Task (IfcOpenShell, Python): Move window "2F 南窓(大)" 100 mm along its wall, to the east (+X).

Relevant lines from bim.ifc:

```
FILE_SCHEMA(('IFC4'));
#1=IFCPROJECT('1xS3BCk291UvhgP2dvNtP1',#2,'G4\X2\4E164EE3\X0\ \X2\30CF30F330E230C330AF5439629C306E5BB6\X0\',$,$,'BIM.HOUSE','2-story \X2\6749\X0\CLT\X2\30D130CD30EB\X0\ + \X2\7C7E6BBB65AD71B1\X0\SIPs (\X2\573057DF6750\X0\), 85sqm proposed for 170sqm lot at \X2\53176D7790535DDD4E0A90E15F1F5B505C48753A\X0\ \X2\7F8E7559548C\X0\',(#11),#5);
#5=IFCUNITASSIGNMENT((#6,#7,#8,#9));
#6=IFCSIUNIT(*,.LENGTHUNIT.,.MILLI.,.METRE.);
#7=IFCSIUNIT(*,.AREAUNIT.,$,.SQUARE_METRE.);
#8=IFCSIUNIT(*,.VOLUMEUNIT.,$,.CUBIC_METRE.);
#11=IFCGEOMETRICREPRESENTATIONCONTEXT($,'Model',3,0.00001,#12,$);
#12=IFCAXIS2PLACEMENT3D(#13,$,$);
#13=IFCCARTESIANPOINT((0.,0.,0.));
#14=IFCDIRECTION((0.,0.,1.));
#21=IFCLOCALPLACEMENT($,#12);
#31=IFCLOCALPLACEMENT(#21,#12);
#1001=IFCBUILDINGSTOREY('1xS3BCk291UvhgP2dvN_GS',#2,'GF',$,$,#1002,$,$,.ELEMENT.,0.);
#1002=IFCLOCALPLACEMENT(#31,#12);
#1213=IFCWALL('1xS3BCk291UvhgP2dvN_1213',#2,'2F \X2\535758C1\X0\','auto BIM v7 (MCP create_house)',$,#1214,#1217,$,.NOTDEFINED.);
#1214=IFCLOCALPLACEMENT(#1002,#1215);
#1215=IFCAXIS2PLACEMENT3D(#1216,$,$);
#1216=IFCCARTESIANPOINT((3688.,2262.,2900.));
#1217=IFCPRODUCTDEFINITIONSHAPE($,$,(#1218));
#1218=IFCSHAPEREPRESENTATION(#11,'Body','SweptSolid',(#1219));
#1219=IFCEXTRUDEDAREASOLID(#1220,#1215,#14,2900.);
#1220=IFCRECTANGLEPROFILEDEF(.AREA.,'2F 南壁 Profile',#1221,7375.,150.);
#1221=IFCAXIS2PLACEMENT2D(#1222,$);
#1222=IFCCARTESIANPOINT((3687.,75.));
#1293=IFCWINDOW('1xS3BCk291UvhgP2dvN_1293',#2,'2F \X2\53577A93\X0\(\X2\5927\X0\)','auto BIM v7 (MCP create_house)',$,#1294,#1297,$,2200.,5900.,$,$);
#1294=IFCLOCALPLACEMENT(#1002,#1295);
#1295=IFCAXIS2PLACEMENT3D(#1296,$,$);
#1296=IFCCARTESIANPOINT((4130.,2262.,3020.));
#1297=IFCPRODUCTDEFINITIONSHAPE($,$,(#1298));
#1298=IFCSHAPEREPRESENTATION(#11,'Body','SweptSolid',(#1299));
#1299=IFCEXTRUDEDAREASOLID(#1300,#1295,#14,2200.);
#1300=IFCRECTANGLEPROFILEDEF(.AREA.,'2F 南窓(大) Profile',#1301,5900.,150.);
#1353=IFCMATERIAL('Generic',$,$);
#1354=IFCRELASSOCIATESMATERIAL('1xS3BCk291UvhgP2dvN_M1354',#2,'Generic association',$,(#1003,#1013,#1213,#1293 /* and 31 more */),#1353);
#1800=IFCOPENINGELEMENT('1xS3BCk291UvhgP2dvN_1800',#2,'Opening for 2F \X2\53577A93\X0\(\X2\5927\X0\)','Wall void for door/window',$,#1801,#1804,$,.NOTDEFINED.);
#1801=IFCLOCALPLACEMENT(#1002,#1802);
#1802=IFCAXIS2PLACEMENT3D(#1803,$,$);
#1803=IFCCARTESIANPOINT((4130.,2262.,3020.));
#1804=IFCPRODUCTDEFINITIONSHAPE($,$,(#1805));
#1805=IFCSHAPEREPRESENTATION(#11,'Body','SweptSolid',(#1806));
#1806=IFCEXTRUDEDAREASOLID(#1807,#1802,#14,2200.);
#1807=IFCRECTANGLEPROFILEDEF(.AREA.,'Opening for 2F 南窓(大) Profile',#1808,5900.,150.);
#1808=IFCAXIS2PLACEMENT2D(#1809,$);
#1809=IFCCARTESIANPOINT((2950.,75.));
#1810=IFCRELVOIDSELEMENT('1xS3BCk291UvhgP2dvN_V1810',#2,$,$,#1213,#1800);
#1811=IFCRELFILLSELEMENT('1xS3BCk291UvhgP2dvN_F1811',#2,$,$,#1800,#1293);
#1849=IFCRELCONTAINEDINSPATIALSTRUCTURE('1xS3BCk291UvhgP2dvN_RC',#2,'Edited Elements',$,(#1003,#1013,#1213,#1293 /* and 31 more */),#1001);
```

```python
import ifcopenshell
import ifcopenshell.api.geometry
import ifcopenshell.util.placement
import ifcopenshell.util.unit

model = ifcopenshell.open("bim.ifc")
unit_scale = ifcopenshell.util.unit.calculate_unit_scale(model)

window = model.by_guid("1xS3BCk291UvhgP2dvN_1293")
opening = window.FillsVoids[0].RelatingOpeningElement
wall = opening.VoidsElements[0].RelatingBuildingElement

wall_matrix = ifcopenshell.util.placement.get_local_placement(wall.ObjectPlacement)
shift = wall_matrix[:3, 0] * 0.1 / unit_scale
before = ifcopenshell.util.placement.get_local_placement(window.ObjectPlacement)[:3, 3].copy()

# The window is not placed relative to its opening, so move both.
for product in (opening, window):
    matrix = ifcopenshell.util.placement.get_local_placement(product.ObjectPlacement)
    matrix[:3, 3] += shift
    ifcopenshell.api.geometry.edit_object_placement(model, product=product, matrix=matrix, is_si=False)

after = ifcopenshell.util.placement.get_local_placement(window.ObjectPlacement)[:3, 3]
print("window moved by", (after - before).round(3) + 0.0)

model.write("bim_rev.ifc")
```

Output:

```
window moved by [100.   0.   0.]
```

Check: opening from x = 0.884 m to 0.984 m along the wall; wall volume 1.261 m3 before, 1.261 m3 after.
